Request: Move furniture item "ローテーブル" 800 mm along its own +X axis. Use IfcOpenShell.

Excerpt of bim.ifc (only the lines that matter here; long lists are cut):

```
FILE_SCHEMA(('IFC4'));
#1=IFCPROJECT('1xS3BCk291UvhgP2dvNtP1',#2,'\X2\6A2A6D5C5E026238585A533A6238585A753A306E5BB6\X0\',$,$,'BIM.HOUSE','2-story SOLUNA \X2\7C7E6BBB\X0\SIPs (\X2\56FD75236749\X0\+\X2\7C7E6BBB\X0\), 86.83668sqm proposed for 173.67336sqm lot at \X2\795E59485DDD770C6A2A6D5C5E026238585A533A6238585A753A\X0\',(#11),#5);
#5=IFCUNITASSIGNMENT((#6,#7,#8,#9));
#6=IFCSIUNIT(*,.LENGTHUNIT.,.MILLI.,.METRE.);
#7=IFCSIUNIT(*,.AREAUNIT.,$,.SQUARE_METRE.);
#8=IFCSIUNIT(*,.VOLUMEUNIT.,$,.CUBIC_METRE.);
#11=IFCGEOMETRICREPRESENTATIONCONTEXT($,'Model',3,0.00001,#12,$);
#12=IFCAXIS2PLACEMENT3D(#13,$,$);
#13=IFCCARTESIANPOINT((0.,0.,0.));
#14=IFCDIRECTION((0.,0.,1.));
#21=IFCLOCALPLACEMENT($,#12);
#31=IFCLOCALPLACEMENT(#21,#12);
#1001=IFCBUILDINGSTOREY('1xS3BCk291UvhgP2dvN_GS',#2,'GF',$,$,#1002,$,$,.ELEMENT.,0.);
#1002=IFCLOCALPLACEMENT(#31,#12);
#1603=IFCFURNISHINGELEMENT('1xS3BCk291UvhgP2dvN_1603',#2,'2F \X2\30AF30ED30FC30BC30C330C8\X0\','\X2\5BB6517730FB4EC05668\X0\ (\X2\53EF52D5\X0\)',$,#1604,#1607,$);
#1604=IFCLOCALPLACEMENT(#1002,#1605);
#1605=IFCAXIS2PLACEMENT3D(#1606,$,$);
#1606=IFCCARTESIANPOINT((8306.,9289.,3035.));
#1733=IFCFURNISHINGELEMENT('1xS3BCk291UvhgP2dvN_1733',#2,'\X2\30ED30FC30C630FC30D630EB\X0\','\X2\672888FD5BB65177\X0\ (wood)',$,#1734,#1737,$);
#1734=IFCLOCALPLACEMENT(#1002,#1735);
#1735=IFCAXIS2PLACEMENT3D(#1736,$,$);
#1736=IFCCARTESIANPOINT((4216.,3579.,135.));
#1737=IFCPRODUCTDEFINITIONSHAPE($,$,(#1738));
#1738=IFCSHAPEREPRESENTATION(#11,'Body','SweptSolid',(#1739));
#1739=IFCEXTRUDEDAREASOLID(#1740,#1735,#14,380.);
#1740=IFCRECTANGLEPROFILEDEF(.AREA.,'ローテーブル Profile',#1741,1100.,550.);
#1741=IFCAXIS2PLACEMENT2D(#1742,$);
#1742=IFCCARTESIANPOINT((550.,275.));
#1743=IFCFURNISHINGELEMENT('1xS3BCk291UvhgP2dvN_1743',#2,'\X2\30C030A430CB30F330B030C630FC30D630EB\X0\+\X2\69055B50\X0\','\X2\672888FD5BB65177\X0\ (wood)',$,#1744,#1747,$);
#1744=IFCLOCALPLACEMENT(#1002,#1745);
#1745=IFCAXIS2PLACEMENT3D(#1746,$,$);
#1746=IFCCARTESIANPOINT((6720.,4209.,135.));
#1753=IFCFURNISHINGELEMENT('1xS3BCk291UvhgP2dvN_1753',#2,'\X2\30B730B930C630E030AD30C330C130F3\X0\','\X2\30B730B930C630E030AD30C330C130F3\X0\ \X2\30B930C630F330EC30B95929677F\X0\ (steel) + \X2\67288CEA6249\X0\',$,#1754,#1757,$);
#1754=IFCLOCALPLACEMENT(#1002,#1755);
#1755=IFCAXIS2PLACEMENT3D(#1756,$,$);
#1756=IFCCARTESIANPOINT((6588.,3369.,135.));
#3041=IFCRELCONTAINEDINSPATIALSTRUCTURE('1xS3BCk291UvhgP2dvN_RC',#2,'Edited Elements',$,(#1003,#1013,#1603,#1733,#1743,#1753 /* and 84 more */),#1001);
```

```python
import ifcopenshell
import ifcopenshell.api.geometry
import ifcopenshell.util.placement
import ifcopenshell.util.unit

model = ifcopenshell.open("bim.ifc")
unit_scale = ifcopenshell.util.unit.calculate_unit_scale(model)

item = model.by_guid("1xS3BCk291UvhgP2dvN_1733")
matrix = ifcopenshell.util.placement.get_local_placement(item.ObjectPlacement)
matrix[:3, 3] += matrix[:3, 0] * 0.8 / unit_scale
ifcopenshell.api.geometry.edit_object_placement(model, product=item, matrix=matrix, is_si=False)

print(ifcopenshell.util.placement.get_local_placement(item.ObjectPlacement).round(3) + 0.0)

model.write("bim-out.ifc")
```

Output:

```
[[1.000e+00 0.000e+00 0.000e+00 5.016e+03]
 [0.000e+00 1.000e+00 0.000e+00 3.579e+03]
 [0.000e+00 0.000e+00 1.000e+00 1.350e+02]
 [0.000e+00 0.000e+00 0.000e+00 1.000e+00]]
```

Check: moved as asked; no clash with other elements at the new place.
